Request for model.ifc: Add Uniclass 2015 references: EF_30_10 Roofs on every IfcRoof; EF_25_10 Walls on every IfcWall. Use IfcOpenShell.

First a look at what the model holds.

```python
import ifcopenshell

model = ifcopenshell.open("model.ifc")
print(model.schema)
print("classifications:", [c.Name for c in model.by_type("IfcClassification")])
for ifc_class in ("IfcDoor", "IfcRoof", "IfcStair", "IfcWall", "IfcWindow"):
    print(ifc_class, len(model.by_type(ifc_class)))
```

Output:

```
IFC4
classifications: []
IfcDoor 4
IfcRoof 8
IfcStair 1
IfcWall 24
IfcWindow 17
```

```python
import ifcopenshell
import ifcopenshell.api.classification

model = ifcopenshell.open("model.ifc")

system = ifcopenshell.api.classification.add_classification(model, classification="Uniclass 2015")

codes = {
    "IfcRoof": ("EF_30_10", "Roofs"),
    "IfcWall": ("EF_25_10", "Walls"),
}
for ifc_class, (code, name) in codes.items():
    products = model.by_type(ifc_class)
    ifcopenshell.api.classification.add_reference(
        model, products=products, classification=system, identification=code, name=name
    )
    print(code, len(products))

model.write("model_rev.ifc")
```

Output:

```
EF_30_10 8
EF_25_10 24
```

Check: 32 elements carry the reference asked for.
